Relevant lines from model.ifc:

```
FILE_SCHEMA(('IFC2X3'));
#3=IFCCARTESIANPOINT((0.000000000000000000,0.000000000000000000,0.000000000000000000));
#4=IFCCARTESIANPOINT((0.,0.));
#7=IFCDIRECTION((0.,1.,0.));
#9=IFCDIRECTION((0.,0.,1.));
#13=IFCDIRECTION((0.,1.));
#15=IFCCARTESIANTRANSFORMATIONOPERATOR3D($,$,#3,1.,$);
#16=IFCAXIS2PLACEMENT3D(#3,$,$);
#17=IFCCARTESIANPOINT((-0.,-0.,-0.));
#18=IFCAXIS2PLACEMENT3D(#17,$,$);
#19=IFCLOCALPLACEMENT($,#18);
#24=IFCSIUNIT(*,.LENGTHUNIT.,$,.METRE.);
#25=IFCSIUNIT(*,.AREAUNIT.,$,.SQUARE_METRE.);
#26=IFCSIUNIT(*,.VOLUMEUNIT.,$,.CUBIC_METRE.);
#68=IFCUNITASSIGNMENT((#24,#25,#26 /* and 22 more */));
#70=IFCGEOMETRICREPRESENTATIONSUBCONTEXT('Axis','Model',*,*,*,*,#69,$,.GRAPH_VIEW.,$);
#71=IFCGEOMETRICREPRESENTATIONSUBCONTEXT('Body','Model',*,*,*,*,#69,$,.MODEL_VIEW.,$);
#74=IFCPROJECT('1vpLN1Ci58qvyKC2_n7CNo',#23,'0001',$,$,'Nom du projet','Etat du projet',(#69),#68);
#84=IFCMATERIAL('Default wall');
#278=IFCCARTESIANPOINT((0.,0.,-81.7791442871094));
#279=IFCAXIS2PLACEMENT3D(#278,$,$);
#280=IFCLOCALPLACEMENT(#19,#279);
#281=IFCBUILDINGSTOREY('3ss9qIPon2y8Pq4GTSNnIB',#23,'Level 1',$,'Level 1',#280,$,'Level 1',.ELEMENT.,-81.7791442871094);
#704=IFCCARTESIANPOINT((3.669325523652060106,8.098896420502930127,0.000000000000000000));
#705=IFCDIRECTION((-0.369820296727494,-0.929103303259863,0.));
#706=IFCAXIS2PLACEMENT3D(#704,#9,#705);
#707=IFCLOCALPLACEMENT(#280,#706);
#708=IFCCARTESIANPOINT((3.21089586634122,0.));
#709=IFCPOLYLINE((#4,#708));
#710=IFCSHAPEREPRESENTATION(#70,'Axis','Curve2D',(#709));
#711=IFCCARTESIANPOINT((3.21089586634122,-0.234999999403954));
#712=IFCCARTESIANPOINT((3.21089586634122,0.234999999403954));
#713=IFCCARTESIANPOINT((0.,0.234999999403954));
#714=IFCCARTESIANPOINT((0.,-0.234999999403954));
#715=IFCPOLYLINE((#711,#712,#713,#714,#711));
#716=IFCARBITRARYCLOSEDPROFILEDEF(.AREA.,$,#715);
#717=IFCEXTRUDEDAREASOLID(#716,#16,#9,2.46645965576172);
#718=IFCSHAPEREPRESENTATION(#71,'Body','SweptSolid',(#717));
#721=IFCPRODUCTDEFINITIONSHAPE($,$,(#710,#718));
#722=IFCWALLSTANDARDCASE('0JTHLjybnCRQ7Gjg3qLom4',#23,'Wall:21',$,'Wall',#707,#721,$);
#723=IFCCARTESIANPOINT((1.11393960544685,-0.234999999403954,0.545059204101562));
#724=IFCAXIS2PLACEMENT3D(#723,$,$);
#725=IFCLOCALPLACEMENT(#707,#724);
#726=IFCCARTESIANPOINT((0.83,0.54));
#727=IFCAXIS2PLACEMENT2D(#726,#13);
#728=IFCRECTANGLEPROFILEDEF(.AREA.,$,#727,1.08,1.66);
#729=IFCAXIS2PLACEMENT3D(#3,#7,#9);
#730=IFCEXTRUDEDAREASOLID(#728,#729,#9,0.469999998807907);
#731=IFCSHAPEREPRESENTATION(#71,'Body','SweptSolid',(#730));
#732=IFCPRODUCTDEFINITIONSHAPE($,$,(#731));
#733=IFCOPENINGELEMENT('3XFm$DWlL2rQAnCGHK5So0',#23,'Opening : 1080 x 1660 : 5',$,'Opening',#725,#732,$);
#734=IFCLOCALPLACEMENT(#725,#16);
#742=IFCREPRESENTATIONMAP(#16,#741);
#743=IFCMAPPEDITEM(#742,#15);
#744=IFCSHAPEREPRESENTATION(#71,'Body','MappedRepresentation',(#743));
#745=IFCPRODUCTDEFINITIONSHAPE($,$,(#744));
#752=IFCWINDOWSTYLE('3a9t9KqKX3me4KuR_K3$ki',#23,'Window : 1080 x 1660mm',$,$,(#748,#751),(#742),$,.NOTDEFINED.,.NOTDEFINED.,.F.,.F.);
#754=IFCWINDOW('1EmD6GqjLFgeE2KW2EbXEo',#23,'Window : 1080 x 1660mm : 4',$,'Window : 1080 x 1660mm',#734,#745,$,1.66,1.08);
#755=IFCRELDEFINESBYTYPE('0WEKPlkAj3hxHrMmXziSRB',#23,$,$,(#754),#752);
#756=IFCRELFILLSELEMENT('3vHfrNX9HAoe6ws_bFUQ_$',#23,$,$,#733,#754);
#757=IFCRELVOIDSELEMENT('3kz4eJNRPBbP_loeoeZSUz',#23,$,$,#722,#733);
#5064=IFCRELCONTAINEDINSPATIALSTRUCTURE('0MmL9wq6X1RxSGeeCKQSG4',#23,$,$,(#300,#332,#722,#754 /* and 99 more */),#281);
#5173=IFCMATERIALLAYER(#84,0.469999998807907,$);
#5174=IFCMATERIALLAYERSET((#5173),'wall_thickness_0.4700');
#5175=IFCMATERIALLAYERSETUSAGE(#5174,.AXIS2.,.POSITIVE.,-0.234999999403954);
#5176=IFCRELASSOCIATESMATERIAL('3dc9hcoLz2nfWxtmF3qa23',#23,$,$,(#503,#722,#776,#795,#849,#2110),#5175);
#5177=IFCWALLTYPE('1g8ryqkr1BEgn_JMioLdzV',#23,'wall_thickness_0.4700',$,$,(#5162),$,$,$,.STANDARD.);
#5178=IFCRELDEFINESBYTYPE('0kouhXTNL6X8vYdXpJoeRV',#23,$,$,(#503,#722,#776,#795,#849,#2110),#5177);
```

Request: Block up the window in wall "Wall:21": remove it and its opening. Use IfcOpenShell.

```python
import ifcopenshell
import ifcopenshell.api.feature
import ifcopenshell.api.root
import ifcopenshell.geom
import ifcopenshell.util.shape

model = ifcopenshell.open("model.ifc")
settings = ifcopenshell.geom.settings()


def volume(element):
    """Net volume in cubic metres, openings subtracted."""
    shape = ifcopenshell.geom.create_shape(settings, element)
    return ifcopenshell.util.shape.get_volume(shape.geometry)


window = model.by_id(754)
opening = window.FillsVoids[0].RelatingOpeningElement
wall = opening.VoidsElements[0].RelatingBuildingElement
before = volume(wall)

ifcopenshell.api.root.remove_product(model, product=window)
ifcopenshell.api.feature.remove_feature(model, feature=opening)

after = volume(wall)

print(f"wall volume {before:.3f} -> {after:.3f} m3")

model.write("model_updated.ifc")
```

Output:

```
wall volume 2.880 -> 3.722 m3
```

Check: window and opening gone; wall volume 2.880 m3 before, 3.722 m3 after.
